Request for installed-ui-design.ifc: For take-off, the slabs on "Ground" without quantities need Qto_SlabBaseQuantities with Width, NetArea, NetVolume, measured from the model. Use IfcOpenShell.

First a look at what the model holds.

```python
import ifcopenshell
import ifcopenshell.util.element
import ifcopenshell.util.unit

model = ifcopenshell.open("installed-ui-design.ifc")
print(model.schema)
for unit_type in ("LENGTHUNIT", "AREAUNIT", "VOLUMEUNIT"):
    print(unit_type, ifcopenshell.util.unit.calculate_unit_scale(model, unit_type))
storey = next(s for s in model.by_type("IfcBuildingStorey") if s.Name == "Ground")
slabs = [e for e in ifcopenshell.util.element.get_decomposition(storey) if e.is_a("IfcSlab")]
for e in sorted(slabs, key=lambda e: e.id()):
    print(e.id(), e.is_a(), e.Name, list(ifcopenshell.util.element.get_psets(e, qtos_only=True)), sep=" | ")
```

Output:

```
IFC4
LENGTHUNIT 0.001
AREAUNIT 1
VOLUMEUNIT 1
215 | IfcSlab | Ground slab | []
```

```python
import ifcopenshell
import ifcopenshell.api.pset
import ifcopenshell.geom
import ifcopenshell.util.element
import ifcopenshell.util.shape
import ifcopenshell.util.unit

model = ifcopenshell.open("installed-ui-design.ifc")
unit_scale = ifcopenshell.util.unit.calculate_unit_scale(model)
area_scale = ifcopenshell.util.unit.calculate_unit_scale(model, "AREAUNIT")
volume_scale = ifcopenshell.util.unit.calculate_unit_scale(model, "VOLUMEUNIT")
settings = ifcopenshell.geom.settings()

storey = next(s for s in model.by_type("IfcBuildingStorey") if s.Name == "Ground")
slabs = [e for e in ifcopenshell.util.element.get_decomposition(storey) if e.is_a("IfcSlab")]

for e in sorted(slabs, key=lambda e: e.id()):
    if ifcopenshell.util.element.get_psets(e, qtos_only=True, should_inherit=False):
        continue
    # Geometry comes back in metres, in the element's own axes.
    shape = ifcopenshell.geom.create_shape(settings, e)
    values = {
        "Width": ifcopenshell.util.shape.get_z(shape.geometry) / unit_scale,
        "NetArea": ifcopenshell.util.shape.get_footprint_area(shape.geometry) / area_scale,
        "NetVolume": ifcopenshell.util.shape.get_volume(shape.geometry) / volume_scale,
    }
    qto = ifcopenshell.api.pset.add_qto(model, product=e, name="Qto_SlabBaseQuantities")
    ifcopenshell.api.pset.edit_qto(model, qto=qto, properties=values)
    print(e.id(), {k: round(v, 3) for k, v in values.items()})

model.write("installed-ui-design-out.ifc")
```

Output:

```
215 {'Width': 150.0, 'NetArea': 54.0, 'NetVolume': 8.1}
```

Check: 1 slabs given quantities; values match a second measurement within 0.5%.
